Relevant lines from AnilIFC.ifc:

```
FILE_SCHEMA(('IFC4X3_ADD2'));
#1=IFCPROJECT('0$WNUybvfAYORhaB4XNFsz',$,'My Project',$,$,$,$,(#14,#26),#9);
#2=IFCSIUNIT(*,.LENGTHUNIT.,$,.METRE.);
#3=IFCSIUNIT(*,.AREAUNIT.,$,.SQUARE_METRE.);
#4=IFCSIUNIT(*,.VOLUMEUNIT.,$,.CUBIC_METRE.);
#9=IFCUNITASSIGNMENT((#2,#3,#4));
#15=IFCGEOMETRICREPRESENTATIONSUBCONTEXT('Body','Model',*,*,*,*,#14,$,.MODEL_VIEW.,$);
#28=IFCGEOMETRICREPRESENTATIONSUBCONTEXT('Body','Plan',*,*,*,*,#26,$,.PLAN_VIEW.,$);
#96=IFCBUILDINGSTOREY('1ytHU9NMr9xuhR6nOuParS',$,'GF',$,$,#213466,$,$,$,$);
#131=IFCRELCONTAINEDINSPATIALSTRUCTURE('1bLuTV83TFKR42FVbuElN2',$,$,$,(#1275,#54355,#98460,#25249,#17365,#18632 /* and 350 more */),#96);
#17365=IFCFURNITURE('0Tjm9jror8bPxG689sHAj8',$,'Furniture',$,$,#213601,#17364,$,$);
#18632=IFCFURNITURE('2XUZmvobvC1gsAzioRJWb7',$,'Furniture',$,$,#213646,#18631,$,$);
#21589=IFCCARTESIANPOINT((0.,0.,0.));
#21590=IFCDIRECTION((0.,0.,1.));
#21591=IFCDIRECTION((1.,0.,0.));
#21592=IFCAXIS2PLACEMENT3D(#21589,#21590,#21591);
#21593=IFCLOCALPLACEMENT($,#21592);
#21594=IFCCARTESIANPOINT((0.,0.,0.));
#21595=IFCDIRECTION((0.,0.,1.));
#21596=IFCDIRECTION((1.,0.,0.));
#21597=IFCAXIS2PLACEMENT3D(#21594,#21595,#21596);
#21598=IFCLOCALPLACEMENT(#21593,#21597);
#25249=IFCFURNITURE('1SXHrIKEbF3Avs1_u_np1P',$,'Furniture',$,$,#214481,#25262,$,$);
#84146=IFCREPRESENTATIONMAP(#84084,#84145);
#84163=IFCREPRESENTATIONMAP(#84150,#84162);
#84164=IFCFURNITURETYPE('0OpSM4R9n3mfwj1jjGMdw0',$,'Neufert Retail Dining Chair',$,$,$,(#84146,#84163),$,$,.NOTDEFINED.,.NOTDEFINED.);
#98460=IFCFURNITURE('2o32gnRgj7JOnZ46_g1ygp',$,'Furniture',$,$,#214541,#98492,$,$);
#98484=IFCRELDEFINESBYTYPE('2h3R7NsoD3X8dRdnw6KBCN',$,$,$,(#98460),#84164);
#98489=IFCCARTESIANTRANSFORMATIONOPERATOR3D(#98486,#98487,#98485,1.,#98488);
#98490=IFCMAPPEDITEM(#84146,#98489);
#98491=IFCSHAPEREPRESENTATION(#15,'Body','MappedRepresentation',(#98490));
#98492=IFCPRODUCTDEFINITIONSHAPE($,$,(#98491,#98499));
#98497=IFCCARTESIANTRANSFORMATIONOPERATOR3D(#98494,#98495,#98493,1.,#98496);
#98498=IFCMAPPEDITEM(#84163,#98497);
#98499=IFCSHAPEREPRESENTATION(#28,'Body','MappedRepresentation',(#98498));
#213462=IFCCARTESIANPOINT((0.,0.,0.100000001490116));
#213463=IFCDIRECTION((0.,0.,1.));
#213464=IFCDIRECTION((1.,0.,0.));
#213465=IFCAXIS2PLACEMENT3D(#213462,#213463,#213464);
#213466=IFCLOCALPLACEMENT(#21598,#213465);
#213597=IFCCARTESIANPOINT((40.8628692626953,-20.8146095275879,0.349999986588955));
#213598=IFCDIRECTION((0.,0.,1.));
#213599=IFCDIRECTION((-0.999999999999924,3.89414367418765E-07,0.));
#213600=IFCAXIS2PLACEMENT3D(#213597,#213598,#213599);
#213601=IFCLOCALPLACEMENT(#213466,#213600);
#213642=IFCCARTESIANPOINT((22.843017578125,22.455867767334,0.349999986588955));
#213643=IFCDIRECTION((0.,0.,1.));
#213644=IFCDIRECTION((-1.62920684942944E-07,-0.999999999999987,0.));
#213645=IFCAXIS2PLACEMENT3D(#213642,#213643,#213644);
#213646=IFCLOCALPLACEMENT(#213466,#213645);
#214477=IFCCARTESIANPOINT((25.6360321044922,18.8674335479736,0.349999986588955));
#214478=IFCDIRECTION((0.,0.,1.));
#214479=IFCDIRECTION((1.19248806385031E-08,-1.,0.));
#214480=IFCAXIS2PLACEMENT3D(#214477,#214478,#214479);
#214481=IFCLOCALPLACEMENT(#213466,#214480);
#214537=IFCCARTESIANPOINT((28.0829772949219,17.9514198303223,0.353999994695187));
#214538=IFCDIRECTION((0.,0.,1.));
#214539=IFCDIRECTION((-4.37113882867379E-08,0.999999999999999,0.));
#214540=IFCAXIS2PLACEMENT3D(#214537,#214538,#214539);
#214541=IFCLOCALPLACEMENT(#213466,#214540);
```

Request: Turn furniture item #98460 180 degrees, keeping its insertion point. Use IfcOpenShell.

```python
import ifcopenshell
import ifcopenshell.api.geometry
import ifcopenshell.util.placement

model = ifcopenshell.open("AnilIFC.ifc")

item = model.by_id(98460)
matrix = ifcopenshell.util.placement.get_local_placement(item.ObjectPlacement)
matrix = matrix @ ifcopenshell.util.placement.rotation(180, "Z")
ifcopenshell.api.geometry.edit_object_placement(model, product=item, matrix=matrix, is_si=False)

print(ifcopenshell.util.placement.get_local_placement(item.ObjectPlacement).round(3) + 0.0)

model.write("AnilIFC_updated.ifc")
```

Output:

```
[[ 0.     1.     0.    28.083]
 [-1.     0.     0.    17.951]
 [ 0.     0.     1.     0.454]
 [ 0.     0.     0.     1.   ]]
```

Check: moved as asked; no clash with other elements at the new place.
